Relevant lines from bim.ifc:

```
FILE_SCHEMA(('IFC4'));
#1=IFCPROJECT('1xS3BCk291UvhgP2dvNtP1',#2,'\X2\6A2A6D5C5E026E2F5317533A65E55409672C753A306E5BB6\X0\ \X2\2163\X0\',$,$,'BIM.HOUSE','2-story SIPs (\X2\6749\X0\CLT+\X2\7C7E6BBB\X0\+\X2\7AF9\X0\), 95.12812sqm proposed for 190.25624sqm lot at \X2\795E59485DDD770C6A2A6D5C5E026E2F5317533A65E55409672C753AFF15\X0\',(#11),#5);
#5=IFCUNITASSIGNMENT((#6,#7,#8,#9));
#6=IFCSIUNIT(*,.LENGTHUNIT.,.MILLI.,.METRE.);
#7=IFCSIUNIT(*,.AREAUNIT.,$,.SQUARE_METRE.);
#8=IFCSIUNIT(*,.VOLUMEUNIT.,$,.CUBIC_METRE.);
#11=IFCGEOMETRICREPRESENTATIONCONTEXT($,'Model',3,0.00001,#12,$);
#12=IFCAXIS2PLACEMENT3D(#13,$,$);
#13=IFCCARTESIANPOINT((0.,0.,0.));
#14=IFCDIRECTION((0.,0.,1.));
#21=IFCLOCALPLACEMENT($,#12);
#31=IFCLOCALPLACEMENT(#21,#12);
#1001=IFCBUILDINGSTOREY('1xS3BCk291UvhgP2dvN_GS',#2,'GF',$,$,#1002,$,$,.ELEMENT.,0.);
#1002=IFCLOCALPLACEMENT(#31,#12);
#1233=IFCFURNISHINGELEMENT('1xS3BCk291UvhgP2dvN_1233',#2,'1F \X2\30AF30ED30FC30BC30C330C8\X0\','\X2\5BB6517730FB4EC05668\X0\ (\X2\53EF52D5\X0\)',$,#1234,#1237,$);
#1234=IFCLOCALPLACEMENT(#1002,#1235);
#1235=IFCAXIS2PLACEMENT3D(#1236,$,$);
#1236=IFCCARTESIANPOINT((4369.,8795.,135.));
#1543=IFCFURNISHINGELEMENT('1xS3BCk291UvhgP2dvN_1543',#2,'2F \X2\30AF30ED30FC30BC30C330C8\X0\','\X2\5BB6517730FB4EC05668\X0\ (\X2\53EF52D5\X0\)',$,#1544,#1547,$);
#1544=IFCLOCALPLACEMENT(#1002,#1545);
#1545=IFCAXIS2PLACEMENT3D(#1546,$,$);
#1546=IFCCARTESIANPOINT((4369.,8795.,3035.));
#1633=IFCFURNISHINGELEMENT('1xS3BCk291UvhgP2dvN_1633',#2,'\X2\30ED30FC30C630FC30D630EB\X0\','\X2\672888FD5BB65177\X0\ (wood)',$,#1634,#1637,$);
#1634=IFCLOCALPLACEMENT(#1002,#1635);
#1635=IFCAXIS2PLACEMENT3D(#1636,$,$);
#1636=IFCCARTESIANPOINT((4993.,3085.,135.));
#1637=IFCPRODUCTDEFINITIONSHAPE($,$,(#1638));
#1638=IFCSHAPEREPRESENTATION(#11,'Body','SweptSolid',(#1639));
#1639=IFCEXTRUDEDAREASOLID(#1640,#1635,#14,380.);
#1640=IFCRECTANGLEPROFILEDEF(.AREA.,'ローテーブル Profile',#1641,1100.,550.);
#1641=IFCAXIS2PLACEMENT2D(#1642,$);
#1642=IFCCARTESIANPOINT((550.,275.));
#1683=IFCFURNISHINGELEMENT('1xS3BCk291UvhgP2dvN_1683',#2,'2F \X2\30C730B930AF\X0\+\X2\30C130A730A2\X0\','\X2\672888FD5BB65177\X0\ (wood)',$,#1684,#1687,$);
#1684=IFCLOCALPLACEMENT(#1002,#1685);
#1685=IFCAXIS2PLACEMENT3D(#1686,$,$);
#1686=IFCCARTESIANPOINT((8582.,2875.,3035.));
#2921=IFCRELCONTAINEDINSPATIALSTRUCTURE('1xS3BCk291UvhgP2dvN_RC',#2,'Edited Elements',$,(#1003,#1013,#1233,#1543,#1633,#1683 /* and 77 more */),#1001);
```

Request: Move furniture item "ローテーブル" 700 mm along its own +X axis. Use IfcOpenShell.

```python
import ifcopenshell
import ifcopenshell.api.geometry
import ifcopenshell.util.placement
import ifcopenshell.util.unit

model = ifcopenshell.open("bim.ifc")
unit_scale = ifcopenshell.util.unit.calculate_unit_scale(model)

item = model.by_guid("1xS3BCk291UvhgP2dvN_1633")
matrix = ifcopenshell.util.placement.get_local_placement(item.ObjectPlacement)
matrix[:3, 3] += matrix[:3, 0] * 0.7 / unit_scale
ifcopenshell.api.geometry.edit_object_placement(model, product=item, matrix=matrix, is_si=False)

print(ifcopenshell.util.placement.get_local_placement(item.ObjectPlacement).round(3) + 0.0)

model.write("bim-out.ifc")
```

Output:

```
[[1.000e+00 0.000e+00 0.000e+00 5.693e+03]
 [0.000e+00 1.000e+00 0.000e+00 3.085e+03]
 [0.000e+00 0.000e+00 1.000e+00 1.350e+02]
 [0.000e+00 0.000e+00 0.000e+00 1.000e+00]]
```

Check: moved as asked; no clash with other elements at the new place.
